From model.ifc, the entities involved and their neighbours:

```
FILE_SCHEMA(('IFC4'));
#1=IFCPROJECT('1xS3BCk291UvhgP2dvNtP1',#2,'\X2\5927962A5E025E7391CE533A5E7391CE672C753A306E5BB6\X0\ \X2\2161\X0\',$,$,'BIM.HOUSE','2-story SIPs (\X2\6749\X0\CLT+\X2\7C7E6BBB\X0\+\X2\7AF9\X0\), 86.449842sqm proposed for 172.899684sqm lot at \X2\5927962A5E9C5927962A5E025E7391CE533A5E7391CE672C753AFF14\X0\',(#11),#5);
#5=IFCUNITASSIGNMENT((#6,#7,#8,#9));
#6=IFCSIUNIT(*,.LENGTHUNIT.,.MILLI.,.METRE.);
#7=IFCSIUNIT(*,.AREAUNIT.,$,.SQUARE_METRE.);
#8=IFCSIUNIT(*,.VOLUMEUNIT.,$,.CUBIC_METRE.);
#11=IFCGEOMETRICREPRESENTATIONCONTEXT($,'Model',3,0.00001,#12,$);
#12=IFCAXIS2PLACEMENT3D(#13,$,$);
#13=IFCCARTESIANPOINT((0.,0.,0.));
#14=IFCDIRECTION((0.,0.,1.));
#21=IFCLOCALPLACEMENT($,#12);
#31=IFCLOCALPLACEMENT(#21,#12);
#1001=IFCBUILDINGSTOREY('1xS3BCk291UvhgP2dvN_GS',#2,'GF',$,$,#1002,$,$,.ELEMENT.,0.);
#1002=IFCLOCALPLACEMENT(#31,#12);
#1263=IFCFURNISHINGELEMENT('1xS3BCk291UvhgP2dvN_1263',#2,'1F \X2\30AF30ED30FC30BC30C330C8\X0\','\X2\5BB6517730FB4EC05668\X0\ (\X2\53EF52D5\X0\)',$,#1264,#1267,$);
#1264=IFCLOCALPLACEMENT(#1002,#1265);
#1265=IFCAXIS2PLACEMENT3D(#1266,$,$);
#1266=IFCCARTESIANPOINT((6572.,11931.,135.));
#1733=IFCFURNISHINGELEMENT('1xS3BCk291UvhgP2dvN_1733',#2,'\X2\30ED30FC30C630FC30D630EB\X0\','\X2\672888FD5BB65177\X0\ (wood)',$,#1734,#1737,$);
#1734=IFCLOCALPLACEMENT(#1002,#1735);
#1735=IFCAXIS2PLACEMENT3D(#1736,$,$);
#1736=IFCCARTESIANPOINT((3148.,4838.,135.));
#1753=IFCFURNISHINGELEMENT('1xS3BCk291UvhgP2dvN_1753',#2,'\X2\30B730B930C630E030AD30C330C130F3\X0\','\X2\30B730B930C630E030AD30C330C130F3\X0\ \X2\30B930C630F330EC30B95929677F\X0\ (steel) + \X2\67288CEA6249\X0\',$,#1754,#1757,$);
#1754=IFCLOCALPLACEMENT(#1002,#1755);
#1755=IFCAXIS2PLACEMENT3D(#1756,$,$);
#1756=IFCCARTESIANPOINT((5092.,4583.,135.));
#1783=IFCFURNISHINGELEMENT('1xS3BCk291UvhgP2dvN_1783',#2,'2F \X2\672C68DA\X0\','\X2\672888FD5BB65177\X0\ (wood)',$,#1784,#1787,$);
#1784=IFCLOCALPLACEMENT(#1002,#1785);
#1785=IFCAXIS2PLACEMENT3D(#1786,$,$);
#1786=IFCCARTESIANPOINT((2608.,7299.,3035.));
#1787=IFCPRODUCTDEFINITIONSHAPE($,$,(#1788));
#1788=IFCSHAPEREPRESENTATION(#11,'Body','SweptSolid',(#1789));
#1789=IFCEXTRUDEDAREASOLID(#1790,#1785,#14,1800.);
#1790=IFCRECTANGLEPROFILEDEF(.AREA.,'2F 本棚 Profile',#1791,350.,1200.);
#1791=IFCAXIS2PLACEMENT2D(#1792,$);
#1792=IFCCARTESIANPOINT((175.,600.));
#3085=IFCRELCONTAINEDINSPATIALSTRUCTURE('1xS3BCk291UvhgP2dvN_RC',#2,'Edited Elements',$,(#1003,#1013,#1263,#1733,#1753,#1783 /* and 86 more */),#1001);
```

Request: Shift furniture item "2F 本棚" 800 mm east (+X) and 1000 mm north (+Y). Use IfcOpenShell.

```python
import ifcopenshell
import ifcopenshell.api.geometry
import ifcopenshell.util.placement
import ifcopenshell.util.unit

model = ifcopenshell.open("model.ifc")
unit_scale = ifcopenshell.util.unit.calculate_unit_scale(model)

item = model.by_guid("1xS3BCk291UvhgP2dvN_1783")
matrix = ifcopenshell.util.placement.get_local_placement(item.ObjectPlacement)
matrix[0, 3] += 0.8 / unit_scale
matrix[1, 3] += 1 / unit_scale
ifcopenshell.api.geometry.edit_object_placement(model, product=item, matrix=matrix, is_si=False)

print(ifcopenshell.util.placement.get_local_placement(item.ObjectPlacement).round(3) + 0.0)

model.write("model_rev.ifc")
```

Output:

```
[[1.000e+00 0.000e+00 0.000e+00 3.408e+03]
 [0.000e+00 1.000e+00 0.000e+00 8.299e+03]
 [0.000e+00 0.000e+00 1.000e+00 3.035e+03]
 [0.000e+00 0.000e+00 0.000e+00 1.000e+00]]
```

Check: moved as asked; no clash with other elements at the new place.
